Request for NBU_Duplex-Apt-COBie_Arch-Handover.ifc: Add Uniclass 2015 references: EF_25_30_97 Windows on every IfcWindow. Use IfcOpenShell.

First a look at what the model holds.

```python
import ifcopenshell

model = ifcopenshell.open("NBU_Duplex-Apt-COBie_Arch-Handover.ifc")
print(model.schema)
print("classifications:", [c.Name for c in model.by_type("IfcClassification")])
for ifc_class in ("IfcDoor", "IfcRoof", "IfcStair", "IfcWall", "IfcWindow"):
    print(ifc_class, len(model.by_type(ifc_class)))
```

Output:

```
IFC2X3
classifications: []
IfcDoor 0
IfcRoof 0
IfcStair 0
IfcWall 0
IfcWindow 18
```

```python
import ifcopenshell
import ifcopenshell.api.classification

model = ifcopenshell.open("NBU_Duplex-Apt-COBie_Arch-Handover.ifc")

# IFC2X3 requires Source and Edition and has no link from the project to the system.
system = model.create_entity("IfcClassification", Source="NBS", Edition="2015", Name="Uniclass 2015")

codes = {
    "IfcWindow": ("EF_25_30_97", "Windows"),
}
for ifc_class, (code, name) in codes.items():
    products = model.by_type(ifc_class)
    ifcopenshell.api.classification.add_reference(
        model, products=products, classification=system, identification=code, name=name
    )
    print(code, len(products))

model.write("NBU_Duplex-Apt-COBie_Arch-Handover-out.ifc")
```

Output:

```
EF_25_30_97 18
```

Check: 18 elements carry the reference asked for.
